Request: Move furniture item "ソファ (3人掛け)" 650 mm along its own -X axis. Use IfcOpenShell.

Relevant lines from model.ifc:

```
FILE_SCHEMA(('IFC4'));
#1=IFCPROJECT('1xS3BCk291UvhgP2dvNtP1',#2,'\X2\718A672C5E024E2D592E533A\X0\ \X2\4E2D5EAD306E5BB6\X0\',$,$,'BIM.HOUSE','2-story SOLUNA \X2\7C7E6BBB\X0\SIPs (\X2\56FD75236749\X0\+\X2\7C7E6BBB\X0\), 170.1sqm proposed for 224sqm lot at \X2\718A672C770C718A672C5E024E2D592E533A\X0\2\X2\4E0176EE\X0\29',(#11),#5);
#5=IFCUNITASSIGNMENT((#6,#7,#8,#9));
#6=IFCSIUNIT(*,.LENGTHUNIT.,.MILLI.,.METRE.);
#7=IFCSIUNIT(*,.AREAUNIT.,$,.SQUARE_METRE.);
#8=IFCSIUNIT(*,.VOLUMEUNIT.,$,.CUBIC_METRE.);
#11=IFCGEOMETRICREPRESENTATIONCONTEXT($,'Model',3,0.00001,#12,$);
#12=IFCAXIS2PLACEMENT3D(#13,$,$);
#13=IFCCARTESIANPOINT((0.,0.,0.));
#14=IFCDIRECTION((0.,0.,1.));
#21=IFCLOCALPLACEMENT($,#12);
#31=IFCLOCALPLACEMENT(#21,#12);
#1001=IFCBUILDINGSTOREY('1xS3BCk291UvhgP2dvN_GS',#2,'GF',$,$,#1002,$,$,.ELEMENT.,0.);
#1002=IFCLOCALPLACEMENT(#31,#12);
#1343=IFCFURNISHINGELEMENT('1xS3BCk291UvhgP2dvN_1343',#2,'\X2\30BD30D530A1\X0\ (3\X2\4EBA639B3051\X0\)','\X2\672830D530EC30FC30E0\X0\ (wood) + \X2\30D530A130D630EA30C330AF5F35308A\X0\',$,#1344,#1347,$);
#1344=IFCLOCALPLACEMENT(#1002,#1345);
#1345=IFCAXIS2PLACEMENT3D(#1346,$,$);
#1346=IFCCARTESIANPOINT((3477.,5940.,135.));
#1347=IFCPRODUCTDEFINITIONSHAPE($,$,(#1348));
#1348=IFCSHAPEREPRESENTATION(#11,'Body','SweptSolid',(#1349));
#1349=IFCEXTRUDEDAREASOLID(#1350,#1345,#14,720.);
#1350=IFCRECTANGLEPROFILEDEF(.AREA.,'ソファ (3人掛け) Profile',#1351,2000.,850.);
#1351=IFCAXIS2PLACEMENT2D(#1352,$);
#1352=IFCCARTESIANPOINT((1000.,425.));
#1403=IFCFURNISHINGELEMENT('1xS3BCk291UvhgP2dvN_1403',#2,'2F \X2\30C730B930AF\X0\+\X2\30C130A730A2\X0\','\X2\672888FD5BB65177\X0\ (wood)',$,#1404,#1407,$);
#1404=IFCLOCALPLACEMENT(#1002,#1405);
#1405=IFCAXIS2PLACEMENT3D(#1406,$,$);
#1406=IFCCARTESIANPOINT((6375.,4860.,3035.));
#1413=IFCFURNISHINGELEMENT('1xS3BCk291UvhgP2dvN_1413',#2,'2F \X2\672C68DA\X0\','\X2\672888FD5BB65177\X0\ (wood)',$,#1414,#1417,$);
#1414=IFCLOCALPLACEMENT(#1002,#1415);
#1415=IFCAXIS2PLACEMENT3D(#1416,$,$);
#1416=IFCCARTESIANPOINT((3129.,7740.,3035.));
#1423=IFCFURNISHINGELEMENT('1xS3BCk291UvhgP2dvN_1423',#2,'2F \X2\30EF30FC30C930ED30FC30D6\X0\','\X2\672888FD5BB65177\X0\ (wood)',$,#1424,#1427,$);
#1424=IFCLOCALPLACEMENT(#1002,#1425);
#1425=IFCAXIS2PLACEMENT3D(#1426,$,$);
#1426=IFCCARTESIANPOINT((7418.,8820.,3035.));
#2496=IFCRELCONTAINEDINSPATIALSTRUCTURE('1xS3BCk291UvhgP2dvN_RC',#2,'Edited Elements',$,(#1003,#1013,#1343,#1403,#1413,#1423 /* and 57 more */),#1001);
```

```python
import ifcopenshell
import ifcopenshell.api.geometry
import ifcopenshell.util.placement

model = ifcopenshell.open("model.ifc")

item = model.by_guid("1xS3BCk291UvhgP2dvN_1343")
matrix = ifcopenshell.util.placement.get_local_placement(item.ObjectPlacement)
matrix[:3, 3] -= matrix[:3, 0] * 650.0
ifcopenshell.api.geometry.edit_object_placement(model, product=item, matrix=matrix, is_si=False)

print(ifcopenshell.util.placement.get_local_placement(item.ObjectPlacement).round(3) + 0.0)

model.write("model_edited.ifc")
```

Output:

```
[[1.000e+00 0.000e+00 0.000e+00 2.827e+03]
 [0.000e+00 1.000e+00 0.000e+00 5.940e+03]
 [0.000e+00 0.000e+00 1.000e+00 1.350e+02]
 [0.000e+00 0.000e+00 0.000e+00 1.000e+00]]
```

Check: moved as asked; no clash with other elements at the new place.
